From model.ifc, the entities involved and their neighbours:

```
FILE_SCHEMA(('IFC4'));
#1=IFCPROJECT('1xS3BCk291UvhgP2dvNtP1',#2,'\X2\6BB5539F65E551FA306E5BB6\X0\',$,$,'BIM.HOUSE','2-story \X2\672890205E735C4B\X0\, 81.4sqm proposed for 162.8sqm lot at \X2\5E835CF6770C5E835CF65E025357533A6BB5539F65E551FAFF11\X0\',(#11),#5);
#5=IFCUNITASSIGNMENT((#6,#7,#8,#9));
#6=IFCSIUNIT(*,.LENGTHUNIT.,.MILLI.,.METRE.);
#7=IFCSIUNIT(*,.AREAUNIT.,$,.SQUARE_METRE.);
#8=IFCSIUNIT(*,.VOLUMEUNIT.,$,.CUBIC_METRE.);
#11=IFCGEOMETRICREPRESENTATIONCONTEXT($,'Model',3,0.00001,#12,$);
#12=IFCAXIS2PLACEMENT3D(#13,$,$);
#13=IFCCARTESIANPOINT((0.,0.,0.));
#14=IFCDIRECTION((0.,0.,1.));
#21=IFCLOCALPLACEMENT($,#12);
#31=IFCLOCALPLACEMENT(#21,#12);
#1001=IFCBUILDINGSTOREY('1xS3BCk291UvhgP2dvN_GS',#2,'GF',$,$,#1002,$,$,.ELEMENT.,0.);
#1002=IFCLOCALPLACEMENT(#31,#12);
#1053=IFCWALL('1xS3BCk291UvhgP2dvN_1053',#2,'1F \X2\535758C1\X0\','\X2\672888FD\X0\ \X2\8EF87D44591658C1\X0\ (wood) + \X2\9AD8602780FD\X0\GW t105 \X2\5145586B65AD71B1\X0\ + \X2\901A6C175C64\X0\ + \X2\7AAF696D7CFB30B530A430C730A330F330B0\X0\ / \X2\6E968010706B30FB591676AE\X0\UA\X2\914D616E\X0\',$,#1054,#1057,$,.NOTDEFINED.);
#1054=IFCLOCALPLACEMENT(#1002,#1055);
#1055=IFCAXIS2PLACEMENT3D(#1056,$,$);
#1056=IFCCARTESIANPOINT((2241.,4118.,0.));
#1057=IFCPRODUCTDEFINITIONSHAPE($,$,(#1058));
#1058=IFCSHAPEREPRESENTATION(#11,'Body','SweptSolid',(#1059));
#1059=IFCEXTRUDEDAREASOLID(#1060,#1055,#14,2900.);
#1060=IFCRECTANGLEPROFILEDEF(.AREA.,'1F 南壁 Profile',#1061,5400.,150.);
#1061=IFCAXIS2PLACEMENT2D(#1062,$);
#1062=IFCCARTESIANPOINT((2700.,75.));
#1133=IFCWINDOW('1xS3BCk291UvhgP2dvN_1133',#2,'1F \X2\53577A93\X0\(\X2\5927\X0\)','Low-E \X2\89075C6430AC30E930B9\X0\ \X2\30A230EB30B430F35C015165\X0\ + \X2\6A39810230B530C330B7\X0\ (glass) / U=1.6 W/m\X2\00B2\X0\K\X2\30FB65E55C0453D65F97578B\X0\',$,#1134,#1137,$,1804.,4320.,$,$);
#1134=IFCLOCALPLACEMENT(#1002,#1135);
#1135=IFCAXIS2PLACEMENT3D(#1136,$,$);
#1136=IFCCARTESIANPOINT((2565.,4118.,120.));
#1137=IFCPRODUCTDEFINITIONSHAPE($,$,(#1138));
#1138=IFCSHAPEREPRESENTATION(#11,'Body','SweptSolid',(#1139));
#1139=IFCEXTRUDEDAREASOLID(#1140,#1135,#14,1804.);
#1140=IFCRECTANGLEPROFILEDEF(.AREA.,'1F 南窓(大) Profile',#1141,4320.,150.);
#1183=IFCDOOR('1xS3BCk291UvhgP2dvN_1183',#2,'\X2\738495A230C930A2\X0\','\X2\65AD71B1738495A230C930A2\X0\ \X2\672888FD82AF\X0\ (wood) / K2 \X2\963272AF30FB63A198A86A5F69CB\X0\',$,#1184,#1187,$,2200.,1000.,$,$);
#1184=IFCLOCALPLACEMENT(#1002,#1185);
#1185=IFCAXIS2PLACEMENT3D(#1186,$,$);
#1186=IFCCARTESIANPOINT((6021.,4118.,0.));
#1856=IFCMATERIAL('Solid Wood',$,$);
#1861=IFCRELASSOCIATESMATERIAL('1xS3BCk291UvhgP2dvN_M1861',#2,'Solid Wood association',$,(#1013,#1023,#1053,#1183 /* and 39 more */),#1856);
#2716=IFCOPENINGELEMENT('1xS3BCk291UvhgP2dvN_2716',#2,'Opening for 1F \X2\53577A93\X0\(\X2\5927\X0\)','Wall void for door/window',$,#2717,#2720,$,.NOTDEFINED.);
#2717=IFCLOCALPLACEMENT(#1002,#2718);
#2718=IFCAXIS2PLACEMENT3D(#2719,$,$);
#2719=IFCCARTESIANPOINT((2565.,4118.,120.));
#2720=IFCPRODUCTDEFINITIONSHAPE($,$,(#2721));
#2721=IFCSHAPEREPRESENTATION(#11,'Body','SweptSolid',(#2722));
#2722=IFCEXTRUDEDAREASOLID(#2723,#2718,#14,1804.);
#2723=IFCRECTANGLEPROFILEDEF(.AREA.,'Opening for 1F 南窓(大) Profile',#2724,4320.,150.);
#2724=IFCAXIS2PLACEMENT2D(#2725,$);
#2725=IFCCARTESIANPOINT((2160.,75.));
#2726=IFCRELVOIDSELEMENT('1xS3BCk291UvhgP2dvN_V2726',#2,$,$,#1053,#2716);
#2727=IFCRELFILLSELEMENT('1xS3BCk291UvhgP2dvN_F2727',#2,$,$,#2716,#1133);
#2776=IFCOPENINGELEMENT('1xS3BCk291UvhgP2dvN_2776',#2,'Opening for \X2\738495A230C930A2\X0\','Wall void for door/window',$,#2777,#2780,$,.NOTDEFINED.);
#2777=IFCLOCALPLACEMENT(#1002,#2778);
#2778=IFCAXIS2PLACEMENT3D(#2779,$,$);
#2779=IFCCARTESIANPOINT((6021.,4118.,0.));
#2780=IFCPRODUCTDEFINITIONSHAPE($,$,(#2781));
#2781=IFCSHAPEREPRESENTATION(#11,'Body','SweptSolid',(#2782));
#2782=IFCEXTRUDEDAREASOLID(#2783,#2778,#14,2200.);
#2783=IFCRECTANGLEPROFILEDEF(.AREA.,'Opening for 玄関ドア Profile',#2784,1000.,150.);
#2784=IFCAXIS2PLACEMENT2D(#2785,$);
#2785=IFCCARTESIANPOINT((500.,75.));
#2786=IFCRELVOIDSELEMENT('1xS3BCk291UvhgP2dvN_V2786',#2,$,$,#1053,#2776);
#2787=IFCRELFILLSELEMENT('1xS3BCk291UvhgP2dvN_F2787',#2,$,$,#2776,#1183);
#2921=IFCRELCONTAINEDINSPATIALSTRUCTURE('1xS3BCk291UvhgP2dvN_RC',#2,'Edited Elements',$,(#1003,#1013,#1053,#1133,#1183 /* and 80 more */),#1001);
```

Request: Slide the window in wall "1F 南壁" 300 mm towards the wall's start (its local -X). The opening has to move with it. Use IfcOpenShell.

```python
import ifcopenshell
import ifcopenshell.api.geometry
import ifcopenshell.util.placement

model = ifcopenshell.open("model.ifc")

window = model.by_guid("1xS3BCk291UvhgP2dvN_1133")
opening = window.FillsVoids[0].RelatingOpeningElement
wall = opening.VoidsElements[0].RelatingBuildingElement

wall_matrix = ifcopenshell.util.placement.get_local_placement(wall.ObjectPlacement)
shift = wall_matrix[:3, 0] * -300.0
before = ifcopenshell.util.placement.get_local_placement(window.ObjectPlacement)[:3, 3].copy()

# The window is not placed relative to its opening, so move both.
for product in (opening, window):
    matrix = ifcopenshell.util.placement.get_local_placement(product.ObjectPlacement)
    matrix[:3, 3] += shift
    ifcopenshell.api.geometry.edit_object_placement(model, product=product, matrix=matrix, is_si=False)

after = ifcopenshell.util.placement.get_local_placement(window.ObjectPlacement)[:3, 3]
print("window moved by", (after - before).round(3) + 0.0)

model.write("model-out.ifc")
```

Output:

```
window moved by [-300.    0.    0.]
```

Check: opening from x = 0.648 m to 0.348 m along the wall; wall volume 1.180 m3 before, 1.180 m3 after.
